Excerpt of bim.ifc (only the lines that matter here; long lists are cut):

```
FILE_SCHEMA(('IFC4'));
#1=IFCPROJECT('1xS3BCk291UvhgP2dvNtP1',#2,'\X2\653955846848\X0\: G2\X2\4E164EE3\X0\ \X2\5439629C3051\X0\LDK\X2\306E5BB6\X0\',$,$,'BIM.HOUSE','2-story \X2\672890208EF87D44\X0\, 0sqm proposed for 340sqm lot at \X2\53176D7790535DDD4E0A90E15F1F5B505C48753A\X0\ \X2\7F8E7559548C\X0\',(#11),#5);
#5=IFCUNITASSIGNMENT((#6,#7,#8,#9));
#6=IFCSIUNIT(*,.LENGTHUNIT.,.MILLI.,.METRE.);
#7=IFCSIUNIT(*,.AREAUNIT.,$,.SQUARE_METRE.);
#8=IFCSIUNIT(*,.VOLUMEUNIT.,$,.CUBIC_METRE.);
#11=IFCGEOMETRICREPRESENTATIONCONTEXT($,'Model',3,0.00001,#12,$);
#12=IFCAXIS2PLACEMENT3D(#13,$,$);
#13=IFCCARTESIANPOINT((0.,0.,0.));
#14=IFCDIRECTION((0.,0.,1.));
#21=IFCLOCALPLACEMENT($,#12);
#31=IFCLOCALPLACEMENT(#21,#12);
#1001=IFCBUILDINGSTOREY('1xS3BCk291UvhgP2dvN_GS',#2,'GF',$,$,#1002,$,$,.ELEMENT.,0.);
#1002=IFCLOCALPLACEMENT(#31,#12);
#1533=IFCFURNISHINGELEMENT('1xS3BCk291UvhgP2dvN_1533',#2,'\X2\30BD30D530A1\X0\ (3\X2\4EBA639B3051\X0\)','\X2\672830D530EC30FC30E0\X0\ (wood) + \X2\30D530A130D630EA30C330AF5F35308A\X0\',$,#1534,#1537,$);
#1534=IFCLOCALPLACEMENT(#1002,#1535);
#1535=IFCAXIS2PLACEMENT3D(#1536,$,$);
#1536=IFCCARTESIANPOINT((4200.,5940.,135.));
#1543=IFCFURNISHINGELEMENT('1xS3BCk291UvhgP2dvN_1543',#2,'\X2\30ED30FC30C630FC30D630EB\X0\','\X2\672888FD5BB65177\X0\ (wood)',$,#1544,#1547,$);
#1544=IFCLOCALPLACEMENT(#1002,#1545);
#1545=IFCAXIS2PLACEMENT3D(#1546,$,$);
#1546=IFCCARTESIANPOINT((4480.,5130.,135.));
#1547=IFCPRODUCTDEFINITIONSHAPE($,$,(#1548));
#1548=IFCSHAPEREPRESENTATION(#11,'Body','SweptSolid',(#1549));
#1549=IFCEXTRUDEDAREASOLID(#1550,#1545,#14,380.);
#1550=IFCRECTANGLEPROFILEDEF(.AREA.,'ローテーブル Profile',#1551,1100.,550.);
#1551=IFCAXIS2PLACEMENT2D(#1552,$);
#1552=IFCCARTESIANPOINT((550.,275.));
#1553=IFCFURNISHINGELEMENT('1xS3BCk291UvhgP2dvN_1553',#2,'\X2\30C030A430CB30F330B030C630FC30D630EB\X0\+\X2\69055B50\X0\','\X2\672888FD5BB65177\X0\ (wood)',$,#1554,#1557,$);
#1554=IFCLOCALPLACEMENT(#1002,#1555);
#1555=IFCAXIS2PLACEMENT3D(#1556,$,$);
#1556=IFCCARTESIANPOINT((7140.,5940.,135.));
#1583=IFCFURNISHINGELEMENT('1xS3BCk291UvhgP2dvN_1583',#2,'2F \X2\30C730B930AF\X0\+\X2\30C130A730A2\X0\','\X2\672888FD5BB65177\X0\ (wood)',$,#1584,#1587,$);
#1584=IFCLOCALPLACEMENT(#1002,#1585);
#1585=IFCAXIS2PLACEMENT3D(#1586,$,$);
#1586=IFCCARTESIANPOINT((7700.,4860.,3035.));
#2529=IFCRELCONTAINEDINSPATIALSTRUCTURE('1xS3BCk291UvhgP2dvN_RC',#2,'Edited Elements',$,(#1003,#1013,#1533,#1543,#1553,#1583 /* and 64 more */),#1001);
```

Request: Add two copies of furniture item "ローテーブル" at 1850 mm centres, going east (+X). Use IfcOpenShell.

```python
import numpy as np
import ifcopenshell
import ifcopenshell.api.geometry
import ifcopenshell.api.root
import ifcopenshell.util.element
import ifcopenshell.util.placement

model = ifcopenshell.open("bim.ifc")


def reuse_history(source, copy):
    """copy_class also copies each property set's owner history, people and application; keep the originals."""
    for rel in copy.IsDefinedBy:
        if rel.is_a("IfcRelDefinesByProperties") and (history := rel.RelatingPropertyDefinition.OwnerHistory):
            rel.RelatingPropertyDefinition.OwnerHistory = source.OwnerHistory
            ifcopenshell.util.element.remove_deep2(model, history)


source = model.by_guid("1xS3BCk291UvhgP2dvN_1543")
base = ifcopenshell.util.placement.get_local_placement(source.ObjectPlacement)
step = np.array([1.0, 0.0, 0.0]) * 1850.0

for i in range(1, 3):
    copy = ifcopenshell.api.root.copy_class(model, product=source)
    copy.Representation = ifcopenshell.util.element.copy_deep(
        model, source.Representation, exclude=["IfcGeometricRepresentationContext", "IfcRepresentationMap"]
    )
    reuse_history(source, copy)
    matrix = base.copy()
    matrix[:3, 3] += i * step
    print("added at", matrix[:3, 3].round(3) + 0.0)
    ifcopenshell.api.geometry.edit_object_placement(model, product=copy, matrix=matrix, is_si=False)

model.write("bim_updated.ifc")
```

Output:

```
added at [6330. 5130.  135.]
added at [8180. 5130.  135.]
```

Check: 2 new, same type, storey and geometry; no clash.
